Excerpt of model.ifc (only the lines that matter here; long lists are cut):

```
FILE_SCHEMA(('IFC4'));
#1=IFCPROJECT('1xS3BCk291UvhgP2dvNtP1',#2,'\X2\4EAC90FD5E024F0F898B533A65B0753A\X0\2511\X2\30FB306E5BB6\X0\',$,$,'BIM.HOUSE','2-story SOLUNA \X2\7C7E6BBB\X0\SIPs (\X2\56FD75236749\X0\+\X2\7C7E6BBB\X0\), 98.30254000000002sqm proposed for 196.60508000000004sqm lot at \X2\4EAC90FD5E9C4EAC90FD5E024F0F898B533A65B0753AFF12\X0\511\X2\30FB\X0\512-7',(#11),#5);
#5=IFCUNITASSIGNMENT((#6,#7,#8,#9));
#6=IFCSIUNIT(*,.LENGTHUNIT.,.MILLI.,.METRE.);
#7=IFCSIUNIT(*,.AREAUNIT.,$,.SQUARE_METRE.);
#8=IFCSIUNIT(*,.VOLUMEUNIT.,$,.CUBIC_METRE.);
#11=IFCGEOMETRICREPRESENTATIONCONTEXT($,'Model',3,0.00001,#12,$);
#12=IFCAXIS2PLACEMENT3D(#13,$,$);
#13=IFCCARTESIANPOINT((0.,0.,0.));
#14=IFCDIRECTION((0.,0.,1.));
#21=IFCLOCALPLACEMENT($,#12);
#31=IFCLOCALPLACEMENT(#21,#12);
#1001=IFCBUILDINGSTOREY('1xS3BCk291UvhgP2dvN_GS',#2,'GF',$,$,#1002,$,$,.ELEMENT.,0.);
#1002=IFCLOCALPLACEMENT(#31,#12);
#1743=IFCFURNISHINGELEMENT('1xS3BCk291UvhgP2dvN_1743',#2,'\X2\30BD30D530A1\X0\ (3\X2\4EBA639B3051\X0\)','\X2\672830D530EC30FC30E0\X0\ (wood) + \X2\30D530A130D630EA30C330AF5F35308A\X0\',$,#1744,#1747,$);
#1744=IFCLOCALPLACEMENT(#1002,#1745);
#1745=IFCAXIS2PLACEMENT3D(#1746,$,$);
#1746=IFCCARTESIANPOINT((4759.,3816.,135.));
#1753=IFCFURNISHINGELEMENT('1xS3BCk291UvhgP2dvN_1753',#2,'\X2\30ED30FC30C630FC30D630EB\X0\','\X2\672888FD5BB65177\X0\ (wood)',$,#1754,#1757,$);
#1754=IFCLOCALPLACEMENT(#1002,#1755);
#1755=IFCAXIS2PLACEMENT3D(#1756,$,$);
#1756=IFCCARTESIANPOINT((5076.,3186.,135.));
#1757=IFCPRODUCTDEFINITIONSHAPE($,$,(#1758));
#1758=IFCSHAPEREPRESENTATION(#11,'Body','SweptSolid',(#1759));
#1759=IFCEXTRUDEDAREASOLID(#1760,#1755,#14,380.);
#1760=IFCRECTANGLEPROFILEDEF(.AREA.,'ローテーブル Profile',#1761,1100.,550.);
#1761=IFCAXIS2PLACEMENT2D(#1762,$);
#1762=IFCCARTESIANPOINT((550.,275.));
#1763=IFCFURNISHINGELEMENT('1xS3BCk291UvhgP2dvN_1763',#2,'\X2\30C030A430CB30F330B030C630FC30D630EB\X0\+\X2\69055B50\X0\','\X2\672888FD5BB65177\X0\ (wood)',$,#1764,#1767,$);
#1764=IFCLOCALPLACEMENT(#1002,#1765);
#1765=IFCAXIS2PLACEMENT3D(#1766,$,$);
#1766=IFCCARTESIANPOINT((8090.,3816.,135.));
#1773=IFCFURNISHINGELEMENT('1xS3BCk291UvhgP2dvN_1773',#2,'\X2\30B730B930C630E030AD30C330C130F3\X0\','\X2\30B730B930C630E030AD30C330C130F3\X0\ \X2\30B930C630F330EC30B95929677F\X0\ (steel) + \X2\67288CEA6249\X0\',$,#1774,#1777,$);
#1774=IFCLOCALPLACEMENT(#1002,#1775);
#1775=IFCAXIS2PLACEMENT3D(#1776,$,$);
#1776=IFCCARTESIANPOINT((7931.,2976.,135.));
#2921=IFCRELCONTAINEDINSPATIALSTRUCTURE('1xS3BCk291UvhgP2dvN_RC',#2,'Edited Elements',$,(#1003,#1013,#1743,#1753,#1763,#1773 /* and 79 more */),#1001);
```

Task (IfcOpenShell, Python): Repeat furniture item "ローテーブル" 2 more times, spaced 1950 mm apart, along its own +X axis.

```python
import ifcopenshell
import ifcopenshell.api.geometry
import ifcopenshell.api.root
import ifcopenshell.util.element
import ifcopenshell.util.placement

model = ifcopenshell.open("model.ifc")


def reuse_history(source, copy):
    """copy_class also copies each property set's owner history, people and application; keep the originals."""
    for rel in copy.IsDefinedBy:
        if rel.is_a("IfcRelDefinesByProperties") and (history := rel.RelatingPropertyDefinition.OwnerHistory):
            rel.RelatingPropertyDefinition.OwnerHistory = source.OwnerHistory
            ifcopenshell.util.element.remove_deep2(model, history)


source = model.by_guid("1xS3BCk291UvhgP2dvN_1753")
base = ifcopenshell.util.placement.get_local_placement(source.ObjectPlacement)
step = base[:3, 0] * 1950.0

for i in range(1, 3):
    copy = ifcopenshell.api.root.copy_class(model, product=source)
    copy.Representation = ifcopenshell.util.element.copy_deep(
        model, source.Representation, exclude=["IfcGeometricRepresentationContext", "IfcRepresentationMap"]
    )
    reuse_history(source, copy)
    matrix = base.copy()
    matrix[:3, 3] += i * step
    print("added at", matrix[:3, 3].round(3) + 0.0)
    ifcopenshell.api.geometry.edit_object_placement(model, product=copy, matrix=matrix, is_si=False)

model.write("model_rev.ifc")
```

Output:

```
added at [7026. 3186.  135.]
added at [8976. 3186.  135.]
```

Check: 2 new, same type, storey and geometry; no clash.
